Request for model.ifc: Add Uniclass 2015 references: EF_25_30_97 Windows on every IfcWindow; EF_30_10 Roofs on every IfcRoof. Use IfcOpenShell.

First a look at what the model holds.

```python
import ifcopenshell

model = ifcopenshell.open("model.ifc")
print(model.schema)
print("classifications:", [c.Name for c in model.by_type("IfcClassification")])
for ifc_class in ("IfcDoor", "IfcRoof", "IfcStair", "IfcWall", "IfcWindow"):
    print(ifc_class, len(model.by_type(ifc_class)))
```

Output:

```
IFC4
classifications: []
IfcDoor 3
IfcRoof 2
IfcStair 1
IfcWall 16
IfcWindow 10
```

```python
import ifcopenshell
import ifcopenshell.api.classification

model = ifcopenshell.open("model.ifc")

system = ifcopenshell.api.classification.add_classification(model, classification="Uniclass 2015")

codes = {
    "IfcWindow": ("EF_25_30_97", "Windows"),
    "IfcRoof": ("EF_30_10", "Roofs"),
}
for ifc_class, (code, name) in codes.items():
    products = model.by_type(ifc_class)
    ifcopenshell.api.classification.add_reference(
        model, products=products, classification=system, identification=code, name=name
    )
    print(code, len(products))

model.write("model_rev.ifc")
```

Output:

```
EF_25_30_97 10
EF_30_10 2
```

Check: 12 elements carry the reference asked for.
